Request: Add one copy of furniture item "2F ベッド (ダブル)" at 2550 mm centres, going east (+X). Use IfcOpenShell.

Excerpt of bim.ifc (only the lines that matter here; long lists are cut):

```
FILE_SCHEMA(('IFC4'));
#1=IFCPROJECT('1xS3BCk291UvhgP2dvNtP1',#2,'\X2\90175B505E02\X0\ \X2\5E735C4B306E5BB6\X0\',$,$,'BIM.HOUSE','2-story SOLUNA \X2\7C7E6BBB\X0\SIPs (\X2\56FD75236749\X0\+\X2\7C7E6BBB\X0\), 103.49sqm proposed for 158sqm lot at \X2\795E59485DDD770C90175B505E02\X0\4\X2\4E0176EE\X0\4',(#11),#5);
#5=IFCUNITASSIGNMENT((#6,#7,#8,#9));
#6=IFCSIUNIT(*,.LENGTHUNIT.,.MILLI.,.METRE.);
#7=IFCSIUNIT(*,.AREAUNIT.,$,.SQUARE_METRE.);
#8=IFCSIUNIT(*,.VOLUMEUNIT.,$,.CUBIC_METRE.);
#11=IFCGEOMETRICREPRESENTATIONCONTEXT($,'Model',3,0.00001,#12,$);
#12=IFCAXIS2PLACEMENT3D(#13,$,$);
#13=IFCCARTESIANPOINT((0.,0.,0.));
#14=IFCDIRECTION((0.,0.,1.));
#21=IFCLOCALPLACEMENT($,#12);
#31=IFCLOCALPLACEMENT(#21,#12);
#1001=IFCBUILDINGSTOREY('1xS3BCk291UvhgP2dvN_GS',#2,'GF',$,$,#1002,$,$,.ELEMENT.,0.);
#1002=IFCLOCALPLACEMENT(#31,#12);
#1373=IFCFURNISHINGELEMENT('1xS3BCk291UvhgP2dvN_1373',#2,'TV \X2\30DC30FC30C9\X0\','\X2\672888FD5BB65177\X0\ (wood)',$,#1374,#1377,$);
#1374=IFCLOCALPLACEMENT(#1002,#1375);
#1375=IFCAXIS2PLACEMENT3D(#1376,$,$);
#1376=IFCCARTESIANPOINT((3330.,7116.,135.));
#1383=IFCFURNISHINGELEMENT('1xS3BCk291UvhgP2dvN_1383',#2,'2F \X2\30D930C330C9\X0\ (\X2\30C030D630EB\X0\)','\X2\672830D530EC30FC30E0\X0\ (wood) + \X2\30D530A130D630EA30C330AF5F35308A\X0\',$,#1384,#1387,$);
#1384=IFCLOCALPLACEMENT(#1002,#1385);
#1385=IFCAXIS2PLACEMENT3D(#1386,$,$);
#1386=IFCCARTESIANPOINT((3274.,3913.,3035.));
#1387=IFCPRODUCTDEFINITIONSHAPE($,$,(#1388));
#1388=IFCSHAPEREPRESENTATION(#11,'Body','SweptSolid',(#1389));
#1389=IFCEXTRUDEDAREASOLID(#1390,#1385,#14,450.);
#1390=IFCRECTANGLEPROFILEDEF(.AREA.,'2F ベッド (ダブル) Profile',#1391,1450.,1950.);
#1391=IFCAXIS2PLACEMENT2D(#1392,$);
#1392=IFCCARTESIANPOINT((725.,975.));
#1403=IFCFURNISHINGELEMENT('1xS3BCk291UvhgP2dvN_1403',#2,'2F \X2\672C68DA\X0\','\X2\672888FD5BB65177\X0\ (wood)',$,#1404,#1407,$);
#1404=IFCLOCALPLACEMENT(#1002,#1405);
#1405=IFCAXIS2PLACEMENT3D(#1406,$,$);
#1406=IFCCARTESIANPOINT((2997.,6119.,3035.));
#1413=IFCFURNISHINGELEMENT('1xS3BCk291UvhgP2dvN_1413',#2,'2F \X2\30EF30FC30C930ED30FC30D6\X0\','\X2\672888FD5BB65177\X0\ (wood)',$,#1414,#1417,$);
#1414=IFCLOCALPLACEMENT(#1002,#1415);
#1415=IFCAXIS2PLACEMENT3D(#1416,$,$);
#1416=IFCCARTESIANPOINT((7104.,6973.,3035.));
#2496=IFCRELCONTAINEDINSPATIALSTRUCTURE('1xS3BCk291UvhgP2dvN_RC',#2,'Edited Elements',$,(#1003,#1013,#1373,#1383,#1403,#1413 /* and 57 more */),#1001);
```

```python
import numpy as np
import ifcopenshell
import ifcopenshell.api.geometry
import ifcopenshell.api.root
import ifcopenshell.util.element
import ifcopenshell.util.placement
import ifcopenshell.util.unit

model = ifcopenshell.open("bim.ifc")
unit_scale = ifcopenshell.util.unit.calculate_unit_scale(model)


def reuse_history(source, copy):
    """copy_class also copies each property set's owner history, people and application; keep the originals."""
    for rel in copy.IsDefinedBy:
        if rel.is_a("IfcRelDefinesByProperties") and (history := rel.RelatingPropertyDefinition.OwnerHistory):
            rel.RelatingPropertyDefinition.OwnerHistory = source.OwnerHistory
            ifcopenshell.util.element.remove_deep2(model, history)


source = model.by_id(1383)
base = ifcopenshell.util.placement.get_local_placement(source.ObjectPlacement)
step = np.array([1.0, 0.0, 0.0]) * 2.55 / unit_scale

for i in range(1, 2):
    copy = ifcopenshell.api.root.copy_class(model, product=source)
    copy.Representation = ifcopenshell.util.element.copy_deep(
        model, source.Representation, exclude=["IfcGeometricRepresentationContext", "IfcRepresentationMap"]
    )
    reuse_history(source, copy)
    matrix = base.copy()
    matrix[:3, 3] += i * step
    print("added at", matrix[:3, 3].round(3) + 0.0)
    ifcopenshell.api.geometry.edit_object_placement(model, product=copy, matrix=matrix, is_si=False)

model.write("bim_rev.ifc")
```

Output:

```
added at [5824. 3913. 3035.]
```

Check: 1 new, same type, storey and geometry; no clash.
